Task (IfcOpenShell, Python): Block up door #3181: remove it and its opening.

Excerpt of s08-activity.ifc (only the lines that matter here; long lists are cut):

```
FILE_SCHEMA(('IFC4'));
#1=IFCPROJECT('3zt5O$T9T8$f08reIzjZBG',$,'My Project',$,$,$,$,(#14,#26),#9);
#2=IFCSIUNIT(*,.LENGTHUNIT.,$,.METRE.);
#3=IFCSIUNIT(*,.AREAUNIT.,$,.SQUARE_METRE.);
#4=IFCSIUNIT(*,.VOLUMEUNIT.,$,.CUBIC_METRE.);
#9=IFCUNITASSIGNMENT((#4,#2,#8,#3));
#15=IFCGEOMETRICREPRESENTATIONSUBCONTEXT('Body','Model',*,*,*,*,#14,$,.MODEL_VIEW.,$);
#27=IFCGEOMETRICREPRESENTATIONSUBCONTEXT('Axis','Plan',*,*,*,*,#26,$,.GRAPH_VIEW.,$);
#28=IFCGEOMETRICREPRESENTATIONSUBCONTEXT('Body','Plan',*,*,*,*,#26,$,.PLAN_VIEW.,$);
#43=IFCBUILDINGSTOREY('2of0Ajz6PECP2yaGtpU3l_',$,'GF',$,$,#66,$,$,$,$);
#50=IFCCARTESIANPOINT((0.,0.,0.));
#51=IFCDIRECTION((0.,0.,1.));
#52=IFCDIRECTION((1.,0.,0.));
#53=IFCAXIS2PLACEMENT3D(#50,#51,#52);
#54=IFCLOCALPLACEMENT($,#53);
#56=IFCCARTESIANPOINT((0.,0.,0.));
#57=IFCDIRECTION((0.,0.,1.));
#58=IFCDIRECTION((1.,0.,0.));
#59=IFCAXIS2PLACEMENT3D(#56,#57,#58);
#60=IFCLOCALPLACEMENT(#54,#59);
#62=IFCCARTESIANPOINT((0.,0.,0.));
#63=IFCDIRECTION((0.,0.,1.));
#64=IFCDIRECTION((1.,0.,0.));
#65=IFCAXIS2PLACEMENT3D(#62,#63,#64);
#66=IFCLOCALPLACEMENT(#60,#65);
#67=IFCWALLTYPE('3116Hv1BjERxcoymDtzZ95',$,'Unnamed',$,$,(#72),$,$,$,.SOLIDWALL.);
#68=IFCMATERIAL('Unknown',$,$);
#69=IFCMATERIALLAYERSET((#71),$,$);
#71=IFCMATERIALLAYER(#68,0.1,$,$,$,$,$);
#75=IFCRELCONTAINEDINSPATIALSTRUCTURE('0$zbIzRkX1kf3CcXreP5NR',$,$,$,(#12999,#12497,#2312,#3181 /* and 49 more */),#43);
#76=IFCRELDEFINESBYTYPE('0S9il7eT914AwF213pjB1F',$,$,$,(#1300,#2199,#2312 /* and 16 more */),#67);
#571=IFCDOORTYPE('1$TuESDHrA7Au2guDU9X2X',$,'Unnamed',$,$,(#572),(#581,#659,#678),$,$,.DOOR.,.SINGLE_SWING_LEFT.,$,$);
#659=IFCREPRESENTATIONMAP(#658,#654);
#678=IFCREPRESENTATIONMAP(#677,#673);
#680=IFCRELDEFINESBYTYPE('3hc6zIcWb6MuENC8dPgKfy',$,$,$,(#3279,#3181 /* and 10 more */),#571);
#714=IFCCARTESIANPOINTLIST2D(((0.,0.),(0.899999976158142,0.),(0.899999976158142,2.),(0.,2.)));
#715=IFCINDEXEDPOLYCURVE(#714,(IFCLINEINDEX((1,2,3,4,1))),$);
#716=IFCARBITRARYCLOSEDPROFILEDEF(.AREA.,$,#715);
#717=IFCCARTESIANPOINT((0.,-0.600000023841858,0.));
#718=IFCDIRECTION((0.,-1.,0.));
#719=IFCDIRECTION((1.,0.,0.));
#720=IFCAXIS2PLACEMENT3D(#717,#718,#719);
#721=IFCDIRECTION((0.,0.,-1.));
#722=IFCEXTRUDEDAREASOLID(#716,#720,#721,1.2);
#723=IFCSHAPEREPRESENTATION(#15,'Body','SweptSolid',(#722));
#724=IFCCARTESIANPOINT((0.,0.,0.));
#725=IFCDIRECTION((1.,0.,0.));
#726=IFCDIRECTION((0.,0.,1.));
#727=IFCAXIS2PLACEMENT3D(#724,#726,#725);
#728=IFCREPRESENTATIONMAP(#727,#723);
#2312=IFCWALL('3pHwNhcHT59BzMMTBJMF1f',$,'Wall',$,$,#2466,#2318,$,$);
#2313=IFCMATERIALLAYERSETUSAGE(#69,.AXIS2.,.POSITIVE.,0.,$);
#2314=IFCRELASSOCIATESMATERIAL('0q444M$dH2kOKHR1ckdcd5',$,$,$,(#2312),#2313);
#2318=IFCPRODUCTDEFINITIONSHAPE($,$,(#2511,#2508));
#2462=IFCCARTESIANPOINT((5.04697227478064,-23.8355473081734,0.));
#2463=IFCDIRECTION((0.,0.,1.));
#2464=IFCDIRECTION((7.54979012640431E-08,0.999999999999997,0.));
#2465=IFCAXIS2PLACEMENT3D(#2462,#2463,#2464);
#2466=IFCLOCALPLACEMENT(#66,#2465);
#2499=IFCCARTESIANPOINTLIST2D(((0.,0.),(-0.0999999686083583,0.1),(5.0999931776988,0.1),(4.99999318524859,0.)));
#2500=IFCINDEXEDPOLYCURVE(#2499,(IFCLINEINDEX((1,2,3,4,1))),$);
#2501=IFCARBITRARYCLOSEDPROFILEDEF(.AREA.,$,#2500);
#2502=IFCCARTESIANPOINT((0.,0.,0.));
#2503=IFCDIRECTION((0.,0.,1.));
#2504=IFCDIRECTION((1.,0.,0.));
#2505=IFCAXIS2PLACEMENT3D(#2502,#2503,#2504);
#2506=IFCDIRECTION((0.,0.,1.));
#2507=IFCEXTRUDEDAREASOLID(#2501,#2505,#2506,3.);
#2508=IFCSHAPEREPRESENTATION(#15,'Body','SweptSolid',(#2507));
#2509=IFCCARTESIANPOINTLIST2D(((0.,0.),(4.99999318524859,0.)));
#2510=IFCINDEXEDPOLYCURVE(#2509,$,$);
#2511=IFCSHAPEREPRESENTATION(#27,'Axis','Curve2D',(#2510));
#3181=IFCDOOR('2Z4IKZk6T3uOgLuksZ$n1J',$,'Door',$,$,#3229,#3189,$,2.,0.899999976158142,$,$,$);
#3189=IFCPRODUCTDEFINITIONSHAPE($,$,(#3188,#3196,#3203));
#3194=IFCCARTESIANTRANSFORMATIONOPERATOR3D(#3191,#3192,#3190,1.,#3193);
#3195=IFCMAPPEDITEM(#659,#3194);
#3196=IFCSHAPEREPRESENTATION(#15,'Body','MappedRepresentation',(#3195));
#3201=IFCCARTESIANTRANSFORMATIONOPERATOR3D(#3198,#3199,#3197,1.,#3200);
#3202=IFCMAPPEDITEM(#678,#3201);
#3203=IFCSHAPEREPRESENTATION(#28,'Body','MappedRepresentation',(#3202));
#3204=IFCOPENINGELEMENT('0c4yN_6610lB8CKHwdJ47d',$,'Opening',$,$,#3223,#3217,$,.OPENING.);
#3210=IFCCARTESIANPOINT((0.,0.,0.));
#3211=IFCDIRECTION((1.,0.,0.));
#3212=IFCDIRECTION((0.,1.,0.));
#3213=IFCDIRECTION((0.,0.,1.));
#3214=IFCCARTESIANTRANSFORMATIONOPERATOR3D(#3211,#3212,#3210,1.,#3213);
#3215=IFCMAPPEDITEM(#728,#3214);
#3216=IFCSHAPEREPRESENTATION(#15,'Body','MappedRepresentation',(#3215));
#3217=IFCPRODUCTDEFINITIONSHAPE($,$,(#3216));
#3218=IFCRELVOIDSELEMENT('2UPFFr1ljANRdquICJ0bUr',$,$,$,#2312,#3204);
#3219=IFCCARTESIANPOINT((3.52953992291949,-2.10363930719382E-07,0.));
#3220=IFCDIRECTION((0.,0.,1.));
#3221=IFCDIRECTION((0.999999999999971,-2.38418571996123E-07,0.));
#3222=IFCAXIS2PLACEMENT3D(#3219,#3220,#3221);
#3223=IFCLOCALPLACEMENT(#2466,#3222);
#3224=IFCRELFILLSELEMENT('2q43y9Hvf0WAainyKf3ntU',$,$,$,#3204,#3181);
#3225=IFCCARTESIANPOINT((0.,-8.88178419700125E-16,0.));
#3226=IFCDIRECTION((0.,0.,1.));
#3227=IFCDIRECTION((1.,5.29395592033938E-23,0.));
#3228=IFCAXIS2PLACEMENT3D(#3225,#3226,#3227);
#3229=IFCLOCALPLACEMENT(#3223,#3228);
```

```python
import ifcopenshell
import ifcopenshell.api.feature
import ifcopenshell.api.root
import ifcopenshell.geom
import ifcopenshell.util.shape

model = ifcopenshell.open("s08-activity.ifc")
settings = ifcopenshell.geom.settings()


def volume(element):
    """Net volume in cubic metres, openings subtracted."""
    shape = ifcopenshell.geom.create_shape(settings, element)
    return ifcopenshell.util.shape.get_volume(shape.geometry)


door = model.by_guid("2Z4IKZk6T3uOgLuksZ$n1J")
opening = door.FillsVoids[0].RelatingOpeningElement
wall = opening.VoidsElements[0].RelatingBuildingElement
before = volume(wall)

ifcopenshell.api.root.remove_product(model, product=door)
ifcopenshell.api.feature.remove_feature(model, feature=opening)

after = volume(wall)

print(f"wall volume {before:.3f} -> {after:.3f} m3")

model.write("s08-activity_rev.ifc")
```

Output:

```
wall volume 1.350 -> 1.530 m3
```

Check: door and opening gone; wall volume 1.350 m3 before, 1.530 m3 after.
